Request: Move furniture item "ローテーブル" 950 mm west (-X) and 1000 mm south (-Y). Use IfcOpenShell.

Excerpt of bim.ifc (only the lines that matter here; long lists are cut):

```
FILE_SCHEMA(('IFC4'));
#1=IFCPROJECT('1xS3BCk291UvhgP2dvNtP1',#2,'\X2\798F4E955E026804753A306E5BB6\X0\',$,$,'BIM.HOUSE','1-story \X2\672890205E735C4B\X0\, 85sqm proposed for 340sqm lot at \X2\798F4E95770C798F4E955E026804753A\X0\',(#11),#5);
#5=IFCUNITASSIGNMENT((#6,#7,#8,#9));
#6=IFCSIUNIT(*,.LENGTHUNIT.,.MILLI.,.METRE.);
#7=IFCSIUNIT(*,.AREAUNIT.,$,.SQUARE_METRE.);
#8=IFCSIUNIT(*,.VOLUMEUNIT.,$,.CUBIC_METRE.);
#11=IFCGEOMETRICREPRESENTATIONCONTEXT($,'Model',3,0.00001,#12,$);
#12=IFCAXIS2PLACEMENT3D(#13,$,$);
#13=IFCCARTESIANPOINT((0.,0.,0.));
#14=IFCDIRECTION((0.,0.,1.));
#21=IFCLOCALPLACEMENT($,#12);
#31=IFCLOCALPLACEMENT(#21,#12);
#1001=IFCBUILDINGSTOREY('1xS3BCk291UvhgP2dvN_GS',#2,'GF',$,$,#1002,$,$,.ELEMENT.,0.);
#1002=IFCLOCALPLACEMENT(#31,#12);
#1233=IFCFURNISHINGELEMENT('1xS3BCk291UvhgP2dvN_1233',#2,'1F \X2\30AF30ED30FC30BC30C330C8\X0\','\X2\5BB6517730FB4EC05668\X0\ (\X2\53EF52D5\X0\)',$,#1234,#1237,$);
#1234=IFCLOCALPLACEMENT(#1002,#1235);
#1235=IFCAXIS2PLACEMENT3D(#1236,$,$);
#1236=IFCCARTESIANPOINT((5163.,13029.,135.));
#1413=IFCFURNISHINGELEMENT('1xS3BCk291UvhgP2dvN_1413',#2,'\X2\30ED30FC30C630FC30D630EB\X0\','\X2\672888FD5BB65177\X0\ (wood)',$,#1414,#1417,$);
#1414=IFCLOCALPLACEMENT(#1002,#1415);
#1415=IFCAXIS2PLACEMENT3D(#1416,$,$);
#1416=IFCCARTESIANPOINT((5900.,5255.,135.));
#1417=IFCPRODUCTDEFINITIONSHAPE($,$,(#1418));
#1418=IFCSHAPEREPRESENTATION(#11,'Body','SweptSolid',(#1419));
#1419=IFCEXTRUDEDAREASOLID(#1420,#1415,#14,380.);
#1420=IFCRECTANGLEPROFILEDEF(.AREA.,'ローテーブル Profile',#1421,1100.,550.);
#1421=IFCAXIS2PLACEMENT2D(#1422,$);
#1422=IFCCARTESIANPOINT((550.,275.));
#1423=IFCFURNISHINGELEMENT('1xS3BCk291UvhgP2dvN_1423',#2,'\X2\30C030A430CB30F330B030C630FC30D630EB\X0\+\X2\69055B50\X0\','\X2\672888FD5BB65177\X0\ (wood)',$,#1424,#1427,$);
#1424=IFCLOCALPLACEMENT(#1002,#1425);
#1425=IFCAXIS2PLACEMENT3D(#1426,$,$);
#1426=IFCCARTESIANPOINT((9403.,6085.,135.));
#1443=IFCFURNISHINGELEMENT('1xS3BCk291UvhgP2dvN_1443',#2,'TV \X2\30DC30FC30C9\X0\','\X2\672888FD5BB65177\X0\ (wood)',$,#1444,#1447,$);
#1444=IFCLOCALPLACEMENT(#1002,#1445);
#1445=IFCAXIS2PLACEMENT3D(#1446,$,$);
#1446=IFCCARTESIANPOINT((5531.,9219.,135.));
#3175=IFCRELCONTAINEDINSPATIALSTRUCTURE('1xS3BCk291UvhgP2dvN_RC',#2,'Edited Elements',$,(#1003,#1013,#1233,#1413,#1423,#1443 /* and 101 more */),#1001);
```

```python
import ifcopenshell
import ifcopenshell.api.geometry
import ifcopenshell.util.placement

model = ifcopenshell.open("bim.ifc")

item = model.by_guid("1xS3BCk291UvhgP2dvN_1413")
matrix = ifcopenshell.util.placement.get_local_placement(item.ObjectPlacement)
matrix[0, 3] -= 950.0
matrix[1, 3] -= 1000.0
ifcopenshell.api.geometry.edit_object_placement(model, product=item, matrix=matrix, is_si=False)

print(ifcopenshell.util.placement.get_local_placement(item.ObjectPlacement).round(3) + 0.0)

model.write("bim_rev.ifc")
```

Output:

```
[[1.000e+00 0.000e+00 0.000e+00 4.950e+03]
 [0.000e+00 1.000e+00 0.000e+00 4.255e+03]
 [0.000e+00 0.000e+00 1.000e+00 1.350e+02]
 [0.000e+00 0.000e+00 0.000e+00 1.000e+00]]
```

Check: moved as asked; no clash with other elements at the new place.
